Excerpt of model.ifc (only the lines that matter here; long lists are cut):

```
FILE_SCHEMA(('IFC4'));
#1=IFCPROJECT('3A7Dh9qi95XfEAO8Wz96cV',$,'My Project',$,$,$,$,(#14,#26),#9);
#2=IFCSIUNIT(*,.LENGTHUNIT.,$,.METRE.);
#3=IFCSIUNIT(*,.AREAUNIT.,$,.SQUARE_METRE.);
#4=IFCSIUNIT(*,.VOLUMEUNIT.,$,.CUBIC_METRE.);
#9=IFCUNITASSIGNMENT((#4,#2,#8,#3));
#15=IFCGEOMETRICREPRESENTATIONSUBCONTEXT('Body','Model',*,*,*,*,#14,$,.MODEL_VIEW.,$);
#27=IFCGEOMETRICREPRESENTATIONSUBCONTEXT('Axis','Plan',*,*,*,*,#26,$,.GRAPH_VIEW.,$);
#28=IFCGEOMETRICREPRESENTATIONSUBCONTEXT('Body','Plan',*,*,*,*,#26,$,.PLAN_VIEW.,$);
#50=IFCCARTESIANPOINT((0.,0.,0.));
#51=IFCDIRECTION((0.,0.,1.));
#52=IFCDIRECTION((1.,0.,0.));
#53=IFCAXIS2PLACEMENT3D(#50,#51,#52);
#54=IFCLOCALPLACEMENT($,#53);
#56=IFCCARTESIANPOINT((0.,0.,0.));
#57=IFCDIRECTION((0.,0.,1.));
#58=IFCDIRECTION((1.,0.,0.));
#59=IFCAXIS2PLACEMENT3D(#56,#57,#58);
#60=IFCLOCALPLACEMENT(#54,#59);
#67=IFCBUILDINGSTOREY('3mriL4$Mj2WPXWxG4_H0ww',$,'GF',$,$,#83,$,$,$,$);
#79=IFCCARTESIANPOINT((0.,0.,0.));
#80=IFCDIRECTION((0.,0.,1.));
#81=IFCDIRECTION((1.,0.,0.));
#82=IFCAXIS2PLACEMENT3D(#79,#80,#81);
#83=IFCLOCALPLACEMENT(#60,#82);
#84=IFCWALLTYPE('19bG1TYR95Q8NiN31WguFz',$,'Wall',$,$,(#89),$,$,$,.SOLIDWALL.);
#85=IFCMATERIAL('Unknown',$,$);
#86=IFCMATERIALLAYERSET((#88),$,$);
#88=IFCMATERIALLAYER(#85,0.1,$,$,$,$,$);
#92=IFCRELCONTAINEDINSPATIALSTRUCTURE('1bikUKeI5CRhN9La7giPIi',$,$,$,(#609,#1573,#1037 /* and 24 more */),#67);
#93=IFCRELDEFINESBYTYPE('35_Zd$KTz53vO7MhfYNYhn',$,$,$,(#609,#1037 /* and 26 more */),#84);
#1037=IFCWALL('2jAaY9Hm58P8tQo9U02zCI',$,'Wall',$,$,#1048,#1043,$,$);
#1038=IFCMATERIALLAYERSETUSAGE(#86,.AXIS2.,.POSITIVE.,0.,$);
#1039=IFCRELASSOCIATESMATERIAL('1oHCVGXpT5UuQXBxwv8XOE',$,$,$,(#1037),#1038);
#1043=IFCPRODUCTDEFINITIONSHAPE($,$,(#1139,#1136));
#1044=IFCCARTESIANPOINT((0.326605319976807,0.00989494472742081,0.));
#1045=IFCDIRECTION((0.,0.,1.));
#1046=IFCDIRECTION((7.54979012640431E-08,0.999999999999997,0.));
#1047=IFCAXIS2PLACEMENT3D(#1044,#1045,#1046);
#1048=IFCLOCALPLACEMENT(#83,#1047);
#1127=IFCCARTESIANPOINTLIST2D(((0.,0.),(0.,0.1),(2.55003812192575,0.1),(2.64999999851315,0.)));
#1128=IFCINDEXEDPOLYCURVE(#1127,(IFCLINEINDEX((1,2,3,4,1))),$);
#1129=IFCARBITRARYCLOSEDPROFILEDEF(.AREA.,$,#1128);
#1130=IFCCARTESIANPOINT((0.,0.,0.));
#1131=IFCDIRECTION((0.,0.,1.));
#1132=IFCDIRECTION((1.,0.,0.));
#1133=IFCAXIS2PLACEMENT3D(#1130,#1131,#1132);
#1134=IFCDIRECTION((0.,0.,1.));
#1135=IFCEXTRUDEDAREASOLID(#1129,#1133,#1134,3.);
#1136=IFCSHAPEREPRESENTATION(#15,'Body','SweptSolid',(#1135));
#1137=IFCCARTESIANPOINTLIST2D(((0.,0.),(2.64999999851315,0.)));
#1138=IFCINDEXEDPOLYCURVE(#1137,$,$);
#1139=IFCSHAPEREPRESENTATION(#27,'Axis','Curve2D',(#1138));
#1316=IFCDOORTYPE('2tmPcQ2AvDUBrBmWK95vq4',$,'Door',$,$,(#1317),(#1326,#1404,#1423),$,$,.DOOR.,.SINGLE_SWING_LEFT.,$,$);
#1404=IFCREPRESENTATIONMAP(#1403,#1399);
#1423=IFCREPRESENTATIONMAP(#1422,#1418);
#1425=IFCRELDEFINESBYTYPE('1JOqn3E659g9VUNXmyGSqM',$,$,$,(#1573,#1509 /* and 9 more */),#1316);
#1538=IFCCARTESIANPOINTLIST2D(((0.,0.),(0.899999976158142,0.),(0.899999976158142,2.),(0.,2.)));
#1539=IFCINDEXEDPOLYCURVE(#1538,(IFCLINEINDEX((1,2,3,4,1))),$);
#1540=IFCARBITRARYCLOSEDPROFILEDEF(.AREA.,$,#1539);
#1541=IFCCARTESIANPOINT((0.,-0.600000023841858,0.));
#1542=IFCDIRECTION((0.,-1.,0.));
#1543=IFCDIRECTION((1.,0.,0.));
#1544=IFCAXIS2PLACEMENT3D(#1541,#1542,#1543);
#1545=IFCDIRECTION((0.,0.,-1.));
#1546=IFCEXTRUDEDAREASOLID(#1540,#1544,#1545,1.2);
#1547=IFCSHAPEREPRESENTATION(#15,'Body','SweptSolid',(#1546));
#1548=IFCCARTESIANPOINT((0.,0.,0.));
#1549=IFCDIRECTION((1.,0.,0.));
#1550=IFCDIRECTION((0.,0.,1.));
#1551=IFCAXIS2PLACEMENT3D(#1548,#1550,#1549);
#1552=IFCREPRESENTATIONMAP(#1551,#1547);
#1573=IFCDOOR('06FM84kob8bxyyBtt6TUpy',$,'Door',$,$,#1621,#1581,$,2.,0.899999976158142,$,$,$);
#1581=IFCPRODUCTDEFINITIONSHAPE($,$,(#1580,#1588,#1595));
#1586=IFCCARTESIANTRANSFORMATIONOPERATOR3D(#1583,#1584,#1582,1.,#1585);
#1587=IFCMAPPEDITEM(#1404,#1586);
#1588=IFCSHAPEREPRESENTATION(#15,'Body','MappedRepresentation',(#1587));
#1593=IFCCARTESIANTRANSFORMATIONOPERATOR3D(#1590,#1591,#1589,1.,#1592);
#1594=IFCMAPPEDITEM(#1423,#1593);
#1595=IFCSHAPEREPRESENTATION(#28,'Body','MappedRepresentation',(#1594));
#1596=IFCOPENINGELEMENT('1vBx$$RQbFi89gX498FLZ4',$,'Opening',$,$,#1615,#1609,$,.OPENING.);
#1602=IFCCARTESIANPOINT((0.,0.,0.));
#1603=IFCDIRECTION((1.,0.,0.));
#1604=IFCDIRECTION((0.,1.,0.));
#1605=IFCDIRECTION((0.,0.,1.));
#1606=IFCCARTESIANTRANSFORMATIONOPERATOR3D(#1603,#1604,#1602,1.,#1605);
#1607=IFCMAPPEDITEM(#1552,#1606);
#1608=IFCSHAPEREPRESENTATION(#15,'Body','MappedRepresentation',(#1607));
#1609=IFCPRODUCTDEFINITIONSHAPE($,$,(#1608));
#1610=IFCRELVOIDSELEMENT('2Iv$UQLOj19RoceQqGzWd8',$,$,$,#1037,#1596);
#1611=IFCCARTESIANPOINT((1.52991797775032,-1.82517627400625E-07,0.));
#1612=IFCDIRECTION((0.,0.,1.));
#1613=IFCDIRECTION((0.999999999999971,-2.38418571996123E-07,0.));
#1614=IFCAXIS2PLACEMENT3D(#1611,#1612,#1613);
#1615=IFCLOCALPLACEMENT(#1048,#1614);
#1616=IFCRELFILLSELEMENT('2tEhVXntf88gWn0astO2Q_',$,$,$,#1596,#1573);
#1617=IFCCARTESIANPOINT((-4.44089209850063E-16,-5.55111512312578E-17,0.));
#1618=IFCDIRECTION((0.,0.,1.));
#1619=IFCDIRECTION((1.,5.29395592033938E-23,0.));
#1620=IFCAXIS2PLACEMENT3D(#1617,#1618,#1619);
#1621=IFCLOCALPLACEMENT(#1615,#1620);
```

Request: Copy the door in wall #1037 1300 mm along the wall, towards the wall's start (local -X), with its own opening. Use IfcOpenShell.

```python
import ifcopenshell
import ifcopenshell.api.feature
import ifcopenshell.api.geometry
import ifcopenshell.api.root
import ifcopenshell.geom
import ifcopenshell.util.element
import ifcopenshell.util.placement
import ifcopenshell.util.shape
import ifcopenshell.util.unit

model = ifcopenshell.open("model.ifc")
unit_scale = ifcopenshell.util.unit.calculate_unit_scale(model)
settings = ifcopenshell.geom.settings()


def volume(element):
    """Net volume in cubic metres, openings subtracted."""
    shape = ifcopenshell.geom.create_shape(settings, element)
    return ifcopenshell.util.shape.get_volume(shape.geometry)


door = model.by_guid("06FM84kob8bxyyBtt6TUpy")
opening = door.FillsVoids[0].RelatingOpeningElement
wall = opening.VoidsElements[0].RelatingBuildingElement
before = volume(wall)
shift = ifcopenshell.util.placement.get_local_placement(wall.ObjectPlacement)[:3, 0] * -1.3 / unit_scale

# copy_class copies the void relationship, type, container and properties, but no geometry.
new_opening = ifcopenshell.api.root.copy_class(model, product=opening)
new_opening.Representation = ifcopenshell.util.element.copy_deep(
    model, opening.Representation, exclude=["IfcGeometricRepresentationContext", "IfcRepresentationMap"]
)
new_door = ifcopenshell.api.root.copy_class(model, product=door)
new_door.Representation = ifcopenshell.util.element.copy_deep(
    model, door.Representation, exclude=["IfcGeometricRepresentationContext", "IfcRepresentationMap"]
)
ifcopenshell.api.feature.add_filling(model, opening=new_opening, element=new_door)

for old, new in ((opening, new_opening), (door, new_door)):
    matrix = ifcopenshell.util.placement.get_local_placement(old.ObjectPlacement)
    matrix[:3, 3] += shift
    ifcopenshell.api.geometry.edit_object_placement(model, product=new, matrix=matrix, is_si=False)

after = volume(wall)

print(f"wall volume {before:.3f} -> {after:.3f} m3")

model.write("model_v2.ifc")
```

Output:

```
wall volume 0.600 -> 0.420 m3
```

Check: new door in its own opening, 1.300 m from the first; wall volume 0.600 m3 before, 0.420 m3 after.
